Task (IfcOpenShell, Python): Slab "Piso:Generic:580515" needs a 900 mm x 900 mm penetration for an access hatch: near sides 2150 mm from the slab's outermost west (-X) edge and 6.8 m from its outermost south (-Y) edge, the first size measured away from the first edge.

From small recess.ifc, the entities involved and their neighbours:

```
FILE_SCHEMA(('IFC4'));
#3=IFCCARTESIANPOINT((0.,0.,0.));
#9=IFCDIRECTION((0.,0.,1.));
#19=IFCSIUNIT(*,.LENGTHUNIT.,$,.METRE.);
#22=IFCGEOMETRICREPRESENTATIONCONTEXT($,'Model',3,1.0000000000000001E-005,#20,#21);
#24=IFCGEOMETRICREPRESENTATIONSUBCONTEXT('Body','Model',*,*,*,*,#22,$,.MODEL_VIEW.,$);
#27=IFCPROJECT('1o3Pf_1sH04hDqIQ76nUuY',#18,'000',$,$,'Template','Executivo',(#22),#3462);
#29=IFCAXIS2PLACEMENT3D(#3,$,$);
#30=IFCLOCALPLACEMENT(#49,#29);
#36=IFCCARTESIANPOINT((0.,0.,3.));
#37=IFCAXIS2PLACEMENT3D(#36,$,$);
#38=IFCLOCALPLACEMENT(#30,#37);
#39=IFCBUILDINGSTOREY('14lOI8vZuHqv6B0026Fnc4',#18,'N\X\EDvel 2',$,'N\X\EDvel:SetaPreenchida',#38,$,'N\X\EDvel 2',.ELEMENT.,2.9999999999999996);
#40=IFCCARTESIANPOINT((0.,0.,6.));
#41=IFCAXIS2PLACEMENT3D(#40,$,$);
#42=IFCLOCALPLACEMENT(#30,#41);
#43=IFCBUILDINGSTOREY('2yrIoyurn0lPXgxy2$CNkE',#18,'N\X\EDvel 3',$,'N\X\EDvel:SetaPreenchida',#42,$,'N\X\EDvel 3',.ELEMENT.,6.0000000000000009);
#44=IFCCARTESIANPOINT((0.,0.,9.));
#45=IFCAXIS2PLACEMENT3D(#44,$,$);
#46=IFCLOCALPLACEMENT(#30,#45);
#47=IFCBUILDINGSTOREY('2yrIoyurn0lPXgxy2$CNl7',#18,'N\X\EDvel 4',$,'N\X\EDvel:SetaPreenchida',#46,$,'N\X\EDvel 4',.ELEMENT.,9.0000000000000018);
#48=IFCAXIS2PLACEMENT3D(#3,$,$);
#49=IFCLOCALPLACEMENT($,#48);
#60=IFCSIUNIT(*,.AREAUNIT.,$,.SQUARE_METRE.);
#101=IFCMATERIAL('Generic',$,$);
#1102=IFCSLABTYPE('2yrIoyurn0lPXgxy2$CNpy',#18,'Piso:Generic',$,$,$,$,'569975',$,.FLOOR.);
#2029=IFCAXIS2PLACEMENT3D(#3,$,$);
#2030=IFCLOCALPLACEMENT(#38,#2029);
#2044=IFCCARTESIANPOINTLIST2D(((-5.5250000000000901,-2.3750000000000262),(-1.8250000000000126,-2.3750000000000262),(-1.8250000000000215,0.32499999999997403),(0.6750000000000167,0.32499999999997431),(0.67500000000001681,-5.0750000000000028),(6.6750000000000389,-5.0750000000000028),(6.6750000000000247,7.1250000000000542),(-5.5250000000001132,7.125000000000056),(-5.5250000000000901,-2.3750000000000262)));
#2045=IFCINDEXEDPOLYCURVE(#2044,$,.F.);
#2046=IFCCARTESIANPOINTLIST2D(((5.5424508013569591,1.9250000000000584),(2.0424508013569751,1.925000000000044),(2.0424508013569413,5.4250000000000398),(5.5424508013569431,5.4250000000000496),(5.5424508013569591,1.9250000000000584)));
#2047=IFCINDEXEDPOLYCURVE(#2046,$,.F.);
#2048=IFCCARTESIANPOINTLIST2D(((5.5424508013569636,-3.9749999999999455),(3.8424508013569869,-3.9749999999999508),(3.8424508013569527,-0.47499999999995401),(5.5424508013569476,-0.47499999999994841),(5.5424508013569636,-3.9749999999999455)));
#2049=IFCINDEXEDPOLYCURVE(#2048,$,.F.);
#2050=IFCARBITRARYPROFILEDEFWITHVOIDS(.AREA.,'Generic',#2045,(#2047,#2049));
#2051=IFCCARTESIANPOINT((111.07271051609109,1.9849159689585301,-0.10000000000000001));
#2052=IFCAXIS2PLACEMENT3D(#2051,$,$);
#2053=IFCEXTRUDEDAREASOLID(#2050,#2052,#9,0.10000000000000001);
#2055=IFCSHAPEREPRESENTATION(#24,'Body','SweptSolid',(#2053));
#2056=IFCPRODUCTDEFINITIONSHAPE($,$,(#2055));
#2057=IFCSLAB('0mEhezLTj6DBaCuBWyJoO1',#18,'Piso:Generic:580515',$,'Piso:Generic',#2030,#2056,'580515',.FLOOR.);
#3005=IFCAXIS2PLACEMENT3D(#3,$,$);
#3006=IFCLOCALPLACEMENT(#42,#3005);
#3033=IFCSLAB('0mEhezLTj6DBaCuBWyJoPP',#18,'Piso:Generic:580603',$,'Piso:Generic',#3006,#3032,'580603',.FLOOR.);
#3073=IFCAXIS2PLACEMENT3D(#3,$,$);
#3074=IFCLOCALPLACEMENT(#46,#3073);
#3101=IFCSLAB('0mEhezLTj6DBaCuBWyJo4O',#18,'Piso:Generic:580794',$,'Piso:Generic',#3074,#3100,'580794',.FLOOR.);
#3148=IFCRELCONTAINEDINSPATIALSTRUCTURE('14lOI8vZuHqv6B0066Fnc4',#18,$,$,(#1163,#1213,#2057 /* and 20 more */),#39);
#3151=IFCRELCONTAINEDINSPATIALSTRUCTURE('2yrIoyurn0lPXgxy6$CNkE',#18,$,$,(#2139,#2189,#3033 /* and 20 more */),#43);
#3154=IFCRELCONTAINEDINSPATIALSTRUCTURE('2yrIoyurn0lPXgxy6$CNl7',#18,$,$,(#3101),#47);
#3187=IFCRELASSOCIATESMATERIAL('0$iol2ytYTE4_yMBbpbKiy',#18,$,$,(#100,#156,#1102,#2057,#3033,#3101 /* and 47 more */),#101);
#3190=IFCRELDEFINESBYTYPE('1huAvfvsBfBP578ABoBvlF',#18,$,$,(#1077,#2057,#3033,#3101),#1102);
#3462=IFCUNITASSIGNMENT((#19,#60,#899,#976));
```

```python
import numpy as np
import ifcopenshell
import ifcopenshell.api.feature
import ifcopenshell.api.geometry
import ifcopenshell.api.root
import ifcopenshell.geom
import ifcopenshell.util.placement
import ifcopenshell.util.representation
import ifcopenshell.util.shape
import ifcopenshell.util.unit

model = ifcopenshell.open("small recess.ifc")
unit_scale = ifcopenshell.util.unit.calculate_unit_scale(model)
settings = ifcopenshell.geom.settings()


def volume(element):
    """Net volume in cubic metres, openings subtracted."""
    shape = ifcopenshell.geom.create_shape(settings, element)
    return ifcopenshell.util.shape.get_volume(shape.geometry)


slab = model.by_guid("0mEhezLTj6DBaCuBWyJoO1")
before = volume(slab)

# Extent in the slab's own axes, in metres. The edges named are its -X and -Y sides.
slab_shape = ifcopenshell.geom.create_shape(settings, slab)
vertices = ifcopenshell.util.shape.get_vertices(slab_shape.geometry)
x_min, y_min, bottom = vertices.min(axis=0)
top = vertices[:, 2].max()

opening = ifcopenshell.api.root.create_entity(model, ifc_class="IfcOpeningElement", name="Access hatch opening", predefined_type="OPENING")
context = ifcopenshell.util.representation.get_context(model, "Model", "Body", "MODEL_VIEW")
width, depth = 0.9, 0.9
outline = [(0.0, 0.0), (width, 0.0), (width, depth), (0.0, depth), (0.0, 0.0)]
# Overshoot both faces by 50 mm so the cut is clean.
shape = ifcopenshell.api.geometry.add_slab_representation(
    model, context=context, depth=top - bottom + 0.1, polyline=outline
)
ifcopenshell.api.geometry.assign_representation(model, product=opening, representation=shape)

matrix = ifcopenshell.util.placement.get_local_placement(slab.ObjectPlacement)
matrix[:, 3] = matrix @ np.append(np.array([x_min + 2.15, y_min + 6.8, bottom - 0.05]) / unit_scale, 1.0)
ifcopenshell.api.geometry.edit_object_placement(model, product=opening, matrix=matrix, is_si=False)
ifcopenshell.api.feature.add_feature(model, feature=opening, element=slab)

after = volume(slab)

print(f"slab volume {before:.3f} -> {after:.3f} m3")

model.write("small recess-out.ifc")
```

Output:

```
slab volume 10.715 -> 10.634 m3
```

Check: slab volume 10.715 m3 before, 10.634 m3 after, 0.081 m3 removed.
